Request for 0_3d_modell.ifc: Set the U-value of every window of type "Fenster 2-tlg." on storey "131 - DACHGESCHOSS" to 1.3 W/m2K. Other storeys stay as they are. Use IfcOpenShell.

First a look at what the model holds.

```python
import ifcopenshell
import ifcopenshell.util.element

model = ifcopenshell.open("0_3d_modell.ifc")
print(model.schema)
storey = next(s for s in model.by_type("IfcBuildingStorey") if s.Name == "131 - DACHGESCHOSS")
windows = [e for e in ifcopenshell.util.element.get_decomposition(storey) if e.is_a("IfcWindow")]
seen = {}
for e in windows:
    element_type = ifcopenshell.util.element.get_type(e)
    key = (element_type.Name if element_type != e and element_type else None, ifcopenshell.util.element.get_pset(e, "Pset_WindowCommon", "ThermalTransmittance"))
    seen[key] = seen.get(key, 0) + 1
for (name, value), count in sorted(seen.items(), key=str):
    print(count, "x", name, "|", value)
```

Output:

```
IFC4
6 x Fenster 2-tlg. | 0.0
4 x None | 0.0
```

```python
import ifcopenshell
import ifcopenshell.api.pset
import ifcopenshell.util.element

model = ifcopenshell.open("0_3d_modell.ifc")

storey = next(s for s in model.by_type("IfcBuildingStorey") if s.Name == "131 - DACHGESCHOSS")
windows = [e for e in ifcopenshell.util.element.get_decomposition(storey) if e.is_a("IfcWindow")]

count = 0
for e in windows:
    element_type = ifcopenshell.util.element.get_type(e)
    if element_type in (None, e) or element_type.Name != "Fenster 2-tlg.":
        continue
    # add_pset returns the element's existing set when there is one.
    pset = ifcopenshell.api.pset.add_pset(model, product=e, name="Pset_WindowCommon")
    ifcopenshell.api.pset.edit_pset(model, pset=pset, properties={"ThermalTransmittance": 1.3})
    count += 1

print(count, "windows updated")

model.write("0_3d_modell-out.ifc")
```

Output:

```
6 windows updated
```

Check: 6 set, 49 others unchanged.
